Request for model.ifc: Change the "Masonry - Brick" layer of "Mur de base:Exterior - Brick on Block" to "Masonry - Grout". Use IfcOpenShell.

First a look at what the model holds.

```python
import ifcopenshell
import ifcopenshell.util.element

model = ifcopenshell.open("model.ifc")
print(model.schema)
for layer_set in model.by_type("IfcMaterialLayerSet"):
    if layer_set.LayerSetName == "Mur de base:Exterior - Brick on Block":
        for layer in layer_set.MaterialLayers:
            print(layer.id(), layer.Material and layer.Material.Name, layer.LayerThickness, sep=" | ")
        print(len(ifcopenshell.util.element.get_elements_by_material(model, layer_set)), "elements and types use it")
print(sorted(m.Name for m in model.by_type("IfcMaterial") if m.Name)[:60])
```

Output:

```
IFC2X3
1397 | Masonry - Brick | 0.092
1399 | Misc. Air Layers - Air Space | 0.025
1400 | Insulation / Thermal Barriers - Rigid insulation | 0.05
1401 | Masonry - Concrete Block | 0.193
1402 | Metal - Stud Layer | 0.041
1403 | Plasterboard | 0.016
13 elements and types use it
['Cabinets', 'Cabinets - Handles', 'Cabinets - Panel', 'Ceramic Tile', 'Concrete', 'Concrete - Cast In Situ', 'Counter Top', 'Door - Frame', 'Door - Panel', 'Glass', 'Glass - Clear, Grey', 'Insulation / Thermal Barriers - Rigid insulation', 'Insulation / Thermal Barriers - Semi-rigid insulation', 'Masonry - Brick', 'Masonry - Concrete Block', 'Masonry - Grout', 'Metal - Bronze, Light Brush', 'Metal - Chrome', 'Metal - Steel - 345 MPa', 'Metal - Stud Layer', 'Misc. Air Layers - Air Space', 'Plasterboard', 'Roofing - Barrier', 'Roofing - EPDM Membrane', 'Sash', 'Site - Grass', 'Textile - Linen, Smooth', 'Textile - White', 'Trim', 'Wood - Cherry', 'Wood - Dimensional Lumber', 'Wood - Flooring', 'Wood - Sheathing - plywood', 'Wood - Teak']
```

```python
import ifcopenshell
import ifcopenshell.api.material

model = ifcopenshell.open("model.ifc")

layer_set = next(s for s in model.by_type("IfcMaterialLayerSet") if s.LayerSetName == "Mur de base:Exterior - Brick on Block")
layer = next(l for l in layer_set.MaterialLayers if l.Material and l.Material.Name == "Masonry - Brick")
material = next(m for m in model.by_type("IfcMaterial") if m.Name == "Masonry - Grout")

# Point this one layer at the other material; renaming the old one would change it everywhere.
ifcopenshell.api.material.edit_layer(model, layer=layer, attributes={}, material=material)

print([l.Material.Name if l.Material else None for l in layer_set.MaterialLayers])

model.write("model_edited.ifc")
```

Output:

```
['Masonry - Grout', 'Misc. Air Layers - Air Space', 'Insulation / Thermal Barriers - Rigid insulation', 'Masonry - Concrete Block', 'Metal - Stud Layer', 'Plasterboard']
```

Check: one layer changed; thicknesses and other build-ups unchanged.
